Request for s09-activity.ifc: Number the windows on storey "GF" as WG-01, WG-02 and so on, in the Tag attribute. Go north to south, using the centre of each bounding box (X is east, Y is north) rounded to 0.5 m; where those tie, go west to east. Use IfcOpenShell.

First a look at what the model holds.

```python
import ifcopenshell
import ifcopenshell.util.element
import ifcopenshell.util.placement

model = ifcopenshell.open("s09-activity.ifc")
print(model.schema)
storey = next(s for s in model.by_type("IfcBuildingStorey") if s.Name == "GF")
windows = [e for e in ifcopenshell.util.element.get_decomposition(storey) if e.is_a("IfcWindow")]
for e in sorted(windows, key=lambda e: e.id()):
    origin = ifcopenshell.util.placement.get_local_placement(e.ObjectPlacement)[:3, 3]
    print(e.id(), e.Tag, e.Name, origin.round(2) + 0.0, sep=" | ")
```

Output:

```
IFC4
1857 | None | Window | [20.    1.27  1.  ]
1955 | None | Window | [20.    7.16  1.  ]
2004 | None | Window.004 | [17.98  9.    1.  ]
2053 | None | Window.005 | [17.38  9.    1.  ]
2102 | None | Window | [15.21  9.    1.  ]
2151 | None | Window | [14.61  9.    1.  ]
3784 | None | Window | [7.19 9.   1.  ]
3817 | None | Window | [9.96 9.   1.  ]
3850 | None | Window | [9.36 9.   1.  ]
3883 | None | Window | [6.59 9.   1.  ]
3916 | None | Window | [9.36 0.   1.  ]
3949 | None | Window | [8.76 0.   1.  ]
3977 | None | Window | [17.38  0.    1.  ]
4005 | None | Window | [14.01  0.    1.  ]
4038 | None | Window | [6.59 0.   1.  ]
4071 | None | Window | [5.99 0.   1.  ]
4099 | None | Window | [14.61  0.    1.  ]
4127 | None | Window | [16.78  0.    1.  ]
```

```python
import ifcopenshell
import ifcopenshell.geom
import ifcopenshell.util.element
import ifcopenshell.util.shape

model = ifcopenshell.open("s09-activity.ifc")
settings = ifcopenshell.geom.settings()
settings.set("use-world-coords", True)


def centre(element):
    shape = ifcopenshell.geom.create_shape(settings, element)
    return ifcopenshell.util.shape.get_bbox_centroid(shape.geometry)


storey = next(s for s in model.by_type("IfcBuildingStorey") if s.Name == "GF")
windows = [e for e in ifcopenshell.util.element.get_decomposition(storey) if e.is_a("IfcWindow")]

# Insertion points can sit at a corner or the storey origin, so sort by the geometry (in metres).
centres = {e: centre(e) for e in windows}
windows.sort(key=lambda e: (-round(centres[e][1] / 0.5), centres[e][0]))

for i, e in enumerate(windows, start=1):
    number = f"WG-{i:02d}"
    e.Tag = number
    print(e.id(), number)

model.write("s09-activity_rev.ifc")
```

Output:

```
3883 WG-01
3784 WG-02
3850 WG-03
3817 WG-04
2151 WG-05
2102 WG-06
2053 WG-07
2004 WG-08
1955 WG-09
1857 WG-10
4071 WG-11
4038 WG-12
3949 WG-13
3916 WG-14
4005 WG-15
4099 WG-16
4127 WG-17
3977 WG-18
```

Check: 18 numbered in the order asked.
